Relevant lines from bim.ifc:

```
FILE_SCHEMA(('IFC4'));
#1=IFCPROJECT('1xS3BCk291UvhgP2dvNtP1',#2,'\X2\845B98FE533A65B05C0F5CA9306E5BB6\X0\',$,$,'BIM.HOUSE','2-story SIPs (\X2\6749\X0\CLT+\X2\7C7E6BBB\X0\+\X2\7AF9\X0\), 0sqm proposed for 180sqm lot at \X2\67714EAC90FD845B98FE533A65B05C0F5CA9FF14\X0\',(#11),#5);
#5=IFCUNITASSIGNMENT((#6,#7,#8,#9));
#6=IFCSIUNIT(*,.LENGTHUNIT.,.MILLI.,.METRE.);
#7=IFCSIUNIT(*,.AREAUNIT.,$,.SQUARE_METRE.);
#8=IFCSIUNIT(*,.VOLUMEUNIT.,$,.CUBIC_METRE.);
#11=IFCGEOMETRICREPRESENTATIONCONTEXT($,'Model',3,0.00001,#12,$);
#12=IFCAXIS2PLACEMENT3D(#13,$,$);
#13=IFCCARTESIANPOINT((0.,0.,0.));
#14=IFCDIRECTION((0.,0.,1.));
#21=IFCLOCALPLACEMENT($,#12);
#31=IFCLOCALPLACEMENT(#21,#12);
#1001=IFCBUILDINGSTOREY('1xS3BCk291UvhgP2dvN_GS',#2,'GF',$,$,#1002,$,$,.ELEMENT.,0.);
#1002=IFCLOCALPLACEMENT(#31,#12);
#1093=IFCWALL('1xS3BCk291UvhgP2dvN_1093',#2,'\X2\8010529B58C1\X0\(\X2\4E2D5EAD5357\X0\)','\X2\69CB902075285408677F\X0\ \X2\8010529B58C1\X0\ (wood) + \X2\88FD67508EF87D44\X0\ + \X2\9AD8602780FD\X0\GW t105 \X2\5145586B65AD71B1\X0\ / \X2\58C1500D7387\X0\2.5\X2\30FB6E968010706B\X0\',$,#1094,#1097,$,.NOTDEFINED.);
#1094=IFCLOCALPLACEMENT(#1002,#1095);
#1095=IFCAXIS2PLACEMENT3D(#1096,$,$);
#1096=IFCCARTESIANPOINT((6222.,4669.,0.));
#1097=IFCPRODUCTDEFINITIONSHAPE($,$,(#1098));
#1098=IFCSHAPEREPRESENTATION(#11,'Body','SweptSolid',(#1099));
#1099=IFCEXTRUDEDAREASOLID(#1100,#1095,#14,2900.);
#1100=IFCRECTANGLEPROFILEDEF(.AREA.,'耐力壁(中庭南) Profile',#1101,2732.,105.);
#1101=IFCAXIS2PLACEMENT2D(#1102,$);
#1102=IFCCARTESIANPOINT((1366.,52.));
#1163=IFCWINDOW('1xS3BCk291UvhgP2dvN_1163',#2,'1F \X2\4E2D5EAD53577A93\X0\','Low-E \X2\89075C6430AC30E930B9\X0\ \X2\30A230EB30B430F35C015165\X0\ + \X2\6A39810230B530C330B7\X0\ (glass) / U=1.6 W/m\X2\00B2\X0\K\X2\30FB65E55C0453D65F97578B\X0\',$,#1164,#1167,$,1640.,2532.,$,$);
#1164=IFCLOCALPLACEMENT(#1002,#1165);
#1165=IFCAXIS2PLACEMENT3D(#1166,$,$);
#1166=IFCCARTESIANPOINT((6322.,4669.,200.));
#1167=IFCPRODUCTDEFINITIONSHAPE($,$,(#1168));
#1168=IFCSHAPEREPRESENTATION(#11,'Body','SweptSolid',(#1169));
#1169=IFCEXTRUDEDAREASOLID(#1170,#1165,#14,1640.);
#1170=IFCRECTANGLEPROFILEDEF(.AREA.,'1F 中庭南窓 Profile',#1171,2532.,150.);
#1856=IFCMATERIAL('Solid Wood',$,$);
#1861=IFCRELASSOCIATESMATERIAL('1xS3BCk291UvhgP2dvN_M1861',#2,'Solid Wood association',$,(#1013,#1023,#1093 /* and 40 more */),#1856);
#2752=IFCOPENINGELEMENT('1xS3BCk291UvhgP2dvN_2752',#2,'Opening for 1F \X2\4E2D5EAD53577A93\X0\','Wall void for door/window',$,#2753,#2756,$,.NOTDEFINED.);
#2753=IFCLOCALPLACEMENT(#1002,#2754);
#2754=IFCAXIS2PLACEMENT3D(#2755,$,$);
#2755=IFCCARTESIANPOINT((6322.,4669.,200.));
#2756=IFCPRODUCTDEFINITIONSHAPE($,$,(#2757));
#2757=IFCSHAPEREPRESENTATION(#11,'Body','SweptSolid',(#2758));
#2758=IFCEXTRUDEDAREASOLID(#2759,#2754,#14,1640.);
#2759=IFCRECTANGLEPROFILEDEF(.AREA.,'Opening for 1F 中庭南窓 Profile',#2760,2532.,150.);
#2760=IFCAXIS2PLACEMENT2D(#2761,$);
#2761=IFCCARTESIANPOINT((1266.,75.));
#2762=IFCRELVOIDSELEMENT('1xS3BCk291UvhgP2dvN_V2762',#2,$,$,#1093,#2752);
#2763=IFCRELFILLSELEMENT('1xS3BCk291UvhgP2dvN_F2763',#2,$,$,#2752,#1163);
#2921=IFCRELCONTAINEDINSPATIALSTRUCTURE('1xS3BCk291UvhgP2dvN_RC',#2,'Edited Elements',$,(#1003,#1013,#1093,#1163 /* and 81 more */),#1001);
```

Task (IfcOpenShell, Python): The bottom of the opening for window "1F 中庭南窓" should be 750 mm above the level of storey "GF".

```python
import numpy as np
import ifcopenshell
import ifcopenshell.api.geometry
import ifcopenshell.geom
import ifcopenshell.util.element
import ifcopenshell.util.placement
import ifcopenshell.util.shape
import ifcopenshell.util.unit

model = ifcopenshell.open("bim.ifc")
unit_scale = ifcopenshell.util.unit.calculate_unit_scale(model)

window = model.by_guid("1xS3BCk291UvhgP2dvN_1163")
opening = window.FillsVoids[0].RelatingOpeningElement
storey = ifcopenshell.util.element.get_container(window, ifc_class="IfcBuildingStorey")
level = ifcopenshell.util.placement.get_local_placement(storey.ObjectPlacement)[2, 3]

# The opening's origin need not be at the sill, so measure its lowest point.
shape = ifcopenshell.geom.create_shape(ifcopenshell.geom.settings(), opening)
bottom = ifcopenshell.util.shape.get_shape_bottom_elevation(shape, shape.geometry) / unit_scale
dz = level + 0.75 / unit_scale - bottom

shift = np.array([0.0, 0.0, dz])
# The window is not placed relative to its opening, so move both.
for product in (opening, window):
    matrix = ifcopenshell.util.placement.get_local_placement(product.ObjectPlacement)
    matrix[:3, 3] += shift
    ifcopenshell.api.geometry.edit_object_placement(model, product=product, matrix=matrix, is_si=False)

print(f"moved by {dz * unit_scale:+.3f} m")

model.write("bim_updated.ifc")
```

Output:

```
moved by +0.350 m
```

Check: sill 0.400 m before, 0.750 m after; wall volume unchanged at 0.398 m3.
